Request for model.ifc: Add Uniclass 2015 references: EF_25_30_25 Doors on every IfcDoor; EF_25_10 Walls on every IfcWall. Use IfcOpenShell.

First a look at what the model holds.

```python
import ifcopenshell

model = ifcopenshell.open("model.ifc")
print(model.schema)
print("classifications:", [c.Name for c in model.by_type("IfcClassification")])
for ifc_class in ("IfcDoor", "IfcRoof", "IfcStair", "IfcWall", "IfcWindow"):
    print(ifc_class, len(model.by_type(ifc_class)))
```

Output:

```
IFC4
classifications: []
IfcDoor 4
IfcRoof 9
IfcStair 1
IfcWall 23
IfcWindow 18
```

```python
import ifcopenshell
import ifcopenshell.api.classification

model = ifcopenshell.open("model.ifc")

system = ifcopenshell.api.classification.add_classification(model, classification="Uniclass 2015")

codes = {
    "IfcDoor": ("EF_25_30_25", "Doors"),
    "IfcWall": ("EF_25_10", "Walls"),
}
for ifc_class, (code, name) in codes.items():
    products = model.by_type(ifc_class)
    ifcopenshell.api.classification.add_reference(
        model, products=products, classification=system, identification=code, name=name
    )
    print(code, len(products))

model.write("model_edited.ifc")
```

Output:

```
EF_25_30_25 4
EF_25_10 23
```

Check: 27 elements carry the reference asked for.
